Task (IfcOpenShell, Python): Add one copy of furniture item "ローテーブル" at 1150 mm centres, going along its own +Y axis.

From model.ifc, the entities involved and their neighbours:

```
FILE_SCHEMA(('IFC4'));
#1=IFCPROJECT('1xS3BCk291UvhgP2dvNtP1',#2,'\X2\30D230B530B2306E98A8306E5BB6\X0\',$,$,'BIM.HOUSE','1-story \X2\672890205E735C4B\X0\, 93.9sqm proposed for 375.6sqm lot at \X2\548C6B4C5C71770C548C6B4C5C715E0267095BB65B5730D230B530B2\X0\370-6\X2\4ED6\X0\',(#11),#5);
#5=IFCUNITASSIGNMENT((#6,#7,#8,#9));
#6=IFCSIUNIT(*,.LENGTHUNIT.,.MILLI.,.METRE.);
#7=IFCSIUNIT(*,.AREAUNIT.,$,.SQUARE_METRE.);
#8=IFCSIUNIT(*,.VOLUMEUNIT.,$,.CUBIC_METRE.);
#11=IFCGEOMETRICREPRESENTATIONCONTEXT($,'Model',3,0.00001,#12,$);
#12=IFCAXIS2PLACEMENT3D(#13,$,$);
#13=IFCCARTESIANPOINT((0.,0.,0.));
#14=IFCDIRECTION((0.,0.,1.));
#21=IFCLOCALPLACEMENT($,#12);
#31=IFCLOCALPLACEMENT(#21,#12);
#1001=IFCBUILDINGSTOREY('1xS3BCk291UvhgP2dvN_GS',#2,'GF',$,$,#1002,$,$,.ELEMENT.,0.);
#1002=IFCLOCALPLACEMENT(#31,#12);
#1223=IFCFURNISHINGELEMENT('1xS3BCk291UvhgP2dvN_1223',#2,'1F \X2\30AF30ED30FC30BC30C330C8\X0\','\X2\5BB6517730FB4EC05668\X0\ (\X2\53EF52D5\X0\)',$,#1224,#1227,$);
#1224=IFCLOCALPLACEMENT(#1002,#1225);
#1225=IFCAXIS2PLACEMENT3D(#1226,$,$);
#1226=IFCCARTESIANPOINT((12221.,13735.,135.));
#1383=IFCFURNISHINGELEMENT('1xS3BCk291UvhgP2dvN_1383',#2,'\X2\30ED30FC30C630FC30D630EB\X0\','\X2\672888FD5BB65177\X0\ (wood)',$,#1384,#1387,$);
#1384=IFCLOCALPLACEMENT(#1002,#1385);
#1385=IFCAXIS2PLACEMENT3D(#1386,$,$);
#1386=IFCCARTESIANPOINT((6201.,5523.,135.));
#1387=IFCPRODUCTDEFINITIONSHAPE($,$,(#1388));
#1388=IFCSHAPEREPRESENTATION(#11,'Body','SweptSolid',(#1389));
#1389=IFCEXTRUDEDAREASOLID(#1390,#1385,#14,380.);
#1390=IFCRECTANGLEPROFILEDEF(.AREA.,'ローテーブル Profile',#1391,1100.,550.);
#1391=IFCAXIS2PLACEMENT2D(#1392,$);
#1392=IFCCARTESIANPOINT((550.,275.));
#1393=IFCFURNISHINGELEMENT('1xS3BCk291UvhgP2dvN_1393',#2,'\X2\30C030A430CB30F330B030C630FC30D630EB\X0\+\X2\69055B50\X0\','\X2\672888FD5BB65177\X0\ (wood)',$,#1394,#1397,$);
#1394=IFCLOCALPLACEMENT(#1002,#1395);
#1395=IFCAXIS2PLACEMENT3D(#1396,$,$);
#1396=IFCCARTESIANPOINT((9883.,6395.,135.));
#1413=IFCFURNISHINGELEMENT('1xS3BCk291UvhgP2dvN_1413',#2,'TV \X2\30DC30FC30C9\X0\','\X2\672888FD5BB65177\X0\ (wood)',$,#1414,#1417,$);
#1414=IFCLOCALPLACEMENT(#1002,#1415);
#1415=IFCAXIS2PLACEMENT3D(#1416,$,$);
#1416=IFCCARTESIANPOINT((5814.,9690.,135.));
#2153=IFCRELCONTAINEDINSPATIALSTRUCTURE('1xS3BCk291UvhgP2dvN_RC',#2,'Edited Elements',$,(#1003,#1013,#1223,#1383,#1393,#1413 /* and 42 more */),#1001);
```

```python
import ifcopenshell
import ifcopenshell.api.geometry
import ifcopenshell.api.root
import ifcopenshell.util.element
import ifcopenshell.util.placement
import ifcopenshell.util.unit

model = ifcopenshell.open("model.ifc")
unit_scale = ifcopenshell.util.unit.calculate_unit_scale(model)


def reuse_history(source, copy):
    """copy_class also copies each property set's owner history, people and application; keep the originals."""
    for rel in copy.IsDefinedBy:
        if rel.is_a("IfcRelDefinesByProperties") and (history := rel.RelatingPropertyDefinition.OwnerHistory):
            rel.RelatingPropertyDefinition.OwnerHistory = source.OwnerHistory
            ifcopenshell.util.element.remove_deep2(model, history)


source = model.by_guid("1xS3BCk291UvhgP2dvN_1383")
base = ifcopenshell.util.placement.get_local_placement(source.ObjectPlacement)
step = base[:3, 1] * 1.15 / unit_scale

for i in range(1, 2):
    copy = ifcopenshell.api.root.copy_class(model, product=source)
    copy.Representation = ifcopenshell.util.element.copy_deep(
        model, source.Representation, exclude=["IfcGeometricRepresentationContext", "IfcRepresentationMap"]
    )
    reuse_history(source, copy)
    matrix = base.copy()
    matrix[:3, 3] += i * step
    print("added at", matrix[:3, 3].round(3) + 0.0)
    ifcopenshell.api.geometry.edit_object_placement(model, product=copy, matrix=matrix, is_si=False)

model.write("model_updated.ifc")
```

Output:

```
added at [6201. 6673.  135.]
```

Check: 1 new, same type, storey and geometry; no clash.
